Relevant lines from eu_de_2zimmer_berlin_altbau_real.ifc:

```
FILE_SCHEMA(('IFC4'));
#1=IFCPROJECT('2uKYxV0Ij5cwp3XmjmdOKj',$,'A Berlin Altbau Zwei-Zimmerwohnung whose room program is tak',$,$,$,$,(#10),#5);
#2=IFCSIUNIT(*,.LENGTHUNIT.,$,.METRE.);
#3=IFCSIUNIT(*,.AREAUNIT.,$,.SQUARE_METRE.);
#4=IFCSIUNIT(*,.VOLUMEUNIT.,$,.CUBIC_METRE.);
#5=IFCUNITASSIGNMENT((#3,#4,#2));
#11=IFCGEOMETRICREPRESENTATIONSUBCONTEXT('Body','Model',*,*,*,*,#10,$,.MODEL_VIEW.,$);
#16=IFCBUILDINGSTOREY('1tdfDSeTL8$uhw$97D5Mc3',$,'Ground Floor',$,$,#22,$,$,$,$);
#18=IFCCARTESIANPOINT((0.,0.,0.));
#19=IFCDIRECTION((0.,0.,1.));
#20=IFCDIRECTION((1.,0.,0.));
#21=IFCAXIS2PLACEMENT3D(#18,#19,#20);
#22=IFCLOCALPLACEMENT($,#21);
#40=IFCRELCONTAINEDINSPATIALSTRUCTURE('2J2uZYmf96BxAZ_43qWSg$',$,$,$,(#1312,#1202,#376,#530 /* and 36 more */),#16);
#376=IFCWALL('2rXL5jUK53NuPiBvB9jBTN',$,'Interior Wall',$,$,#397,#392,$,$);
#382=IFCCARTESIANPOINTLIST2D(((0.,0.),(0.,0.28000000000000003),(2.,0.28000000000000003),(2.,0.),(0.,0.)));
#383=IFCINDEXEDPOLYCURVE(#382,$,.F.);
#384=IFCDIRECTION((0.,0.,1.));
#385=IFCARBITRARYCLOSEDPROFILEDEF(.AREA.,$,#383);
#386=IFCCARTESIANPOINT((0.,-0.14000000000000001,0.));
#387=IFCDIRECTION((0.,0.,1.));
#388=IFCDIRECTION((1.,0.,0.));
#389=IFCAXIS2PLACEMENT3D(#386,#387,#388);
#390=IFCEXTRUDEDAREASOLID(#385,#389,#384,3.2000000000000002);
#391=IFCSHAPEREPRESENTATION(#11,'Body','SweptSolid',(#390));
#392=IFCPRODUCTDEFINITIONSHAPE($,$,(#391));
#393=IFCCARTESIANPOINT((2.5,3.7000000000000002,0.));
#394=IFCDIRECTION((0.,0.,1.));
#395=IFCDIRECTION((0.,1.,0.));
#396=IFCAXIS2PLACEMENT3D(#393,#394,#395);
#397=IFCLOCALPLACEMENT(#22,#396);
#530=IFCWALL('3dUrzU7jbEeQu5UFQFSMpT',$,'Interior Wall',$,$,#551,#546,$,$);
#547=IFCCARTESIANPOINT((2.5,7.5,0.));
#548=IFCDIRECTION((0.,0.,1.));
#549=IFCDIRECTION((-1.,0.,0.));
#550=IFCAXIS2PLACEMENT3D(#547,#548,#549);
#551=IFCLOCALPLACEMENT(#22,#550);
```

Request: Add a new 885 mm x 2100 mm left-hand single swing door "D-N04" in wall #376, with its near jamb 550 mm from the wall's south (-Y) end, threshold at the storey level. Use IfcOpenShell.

```python
import numpy as np
import ifcopenshell
import ifcopenshell.api.feature
import ifcopenshell.api.geometry
import ifcopenshell.api.root
import ifcopenshell.api.spatial
import ifcopenshell.geom
import ifcopenshell.util.element
import ifcopenshell.util.placement
import ifcopenshell.util.representation
import ifcopenshell.util.shape
import ifcopenshell.util.unit

model = ifcopenshell.open("eu_de_2zimmer_berlin_altbau_real.ifc")
unit_scale = ifcopenshell.util.unit.calculate_unit_scale(model)
settings = ifcopenshell.geom.settings()


def volume(element):
    """Net volume in cubic metres, openings subtracted."""
    shape = ifcopenshell.geom.create_shape(settings, element)
    return ifcopenshell.util.shape.get_volume(shape.geometry)


wall = model.by_guid("2rXL5jUK53NuPiBvB9jBTN")
storey = ifcopenshell.util.element.get_container(wall, ifc_class="IfcBuildingStorey")
context = ifcopenshell.util.representation.get_context(model, "Model", "Body", "MODEL_VIEW")
before = volume(wall)

width, height, from_end, sill = 0.885, 2.1, 0.55, 0.0  # metres

# The wall runs along its own X axis, and the end named is its -X end.
wall_shape = ifcopenshell.geom.create_shape(settings, wall)
x, y, z = ifcopenshell.util.shape.get_vertices(wall_shape.geometry).T
start = x.min() + from_end
face, thickness = float(y.min()), float(y.max() - y.min())
wall_matrix = ifcopenshell.util.placement.get_local_placement(wall.ObjectPlacement)
level = ifcopenshell.util.placement.get_local_placement(storey.ObjectPlacement)[2, 3]


def in_wall(x, y):
    """Placement at x, y metres in the wall's axes, at sill height."""
    matrix = wall_matrix.copy()
    matrix[:, 3] = wall_matrix @ np.array([x / unit_scale, y / unit_scale, 0.0, 1.0])
    matrix[2, 3] = level + sill / unit_scale
    return matrix


# Opening: a box that overshoots both wall faces by 50 mm.
opening = ifcopenshell.api.root.create_entity(model, ifc_class="IfcOpeningElement", predefined_type="OPENING")
box = ifcopenshell.api.geometry.add_wall_representation(
    model, context=context, length=width, height=height, thickness=thickness + 0.1
)
ifcopenshell.api.geometry.assign_representation(model, product=opening, representation=box)
ifcopenshell.api.geometry.edit_object_placement(model, product=opening, matrix=in_wall(start, face - 0.05), is_si=False)
ifcopenshell.api.feature.add_feature(model, feature=opening, element=wall)

door = ifcopenshell.api.root.create_entity(model, ifc_class="IfcDoor", name="D-N04", predefined_type="DOOR")
door.OverallWidth, door.OverallHeight = width / unit_scale, height / unit_scale
door.OperationType = "SINGLE_SWING_LEFT"
body = ifcopenshell.api.geometry.add_door_representation(
    model,
    context=context,
    overall_width=door.OverallWidth,
    overall_height=door.OverallHeight,
    operation_type="SINGLE_SWING_LEFT",
    lining_properties={"LiningDepth": thickness / unit_scale, "ThresholdDepth": thickness / unit_scale},
)
ifcopenshell.api.geometry.assign_representation(model, product=door, representation=body)
ifcopenshell.api.spatial.assign_container(model, products=[door], relating_structure=storey)
ifcopenshell.api.feature.add_filling(model, opening=opening, element=door)

# The lining spans the wall, so the door starts at the wall face.
ifcopenshell.api.geometry.edit_object_placement(model, product=door, matrix=in_wall(start, face), is_si=False)

after = volume(wall)

print(f"wall volume {before:.3f} -> {after:.3f} m3")

model.write("eu_de_2zimmer_berlin_altbau_real_updated.ifc")
```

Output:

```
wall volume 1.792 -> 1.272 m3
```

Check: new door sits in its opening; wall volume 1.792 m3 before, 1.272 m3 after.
